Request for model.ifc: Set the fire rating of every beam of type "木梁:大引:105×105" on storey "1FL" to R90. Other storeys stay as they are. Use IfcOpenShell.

First a look at what the model holds.

```python
import ifcopenshell
import ifcopenshell.util.element

model = ifcopenshell.open("model.ifc")
print(model.schema)
storey = next(s for s in model.by_type("IfcBuildingStorey") if s.Name == "1FL")
beams = [e for e in ifcopenshell.util.element.get_decomposition(storey) if e.is_a("IfcBeam")]
seen = {}
for e in beams:
    element_type = ifcopenshell.util.element.get_type(e)
    key = (element_type.Name if element_type != e and element_type else None, ifcopenshell.util.element.get_pset(e, "Pset_BeamCommon", "FireRating"))
    seen[key] = seen.get(key, 0) + 1
for (name, value), count in sorted(seen.items(), key=str):
    print(count, "x", name, "|", value)
```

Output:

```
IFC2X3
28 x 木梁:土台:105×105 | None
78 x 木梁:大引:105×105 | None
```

```python
import ifcopenshell
import ifcopenshell.api.pset
import ifcopenshell.util.element

model = ifcopenshell.open("model.ifc")

storey = next(s for s in model.by_type("IfcBuildingStorey") if s.Name == "1FL")
beams = [e for e in ifcopenshell.util.element.get_decomposition(storey) if e.is_a("IfcBeam")]

count = 0
for e in beams:
    element_type = ifcopenshell.util.element.get_type(e)
    if element_type in (None, e) or element_type.Name != "木梁:大引:105×105":
        continue
    # add_pset returns the element's existing set when there is one.
    pset = ifcopenshell.api.pset.add_pset(model, product=e, name="Pset_BeamCommon")
    ifcopenshell.api.pset.edit_pset(model, pset=pset, properties={"FireRating": "R90"})
    count += 1

print(count, "beams updated")

model.write("model_v2.ifc")
```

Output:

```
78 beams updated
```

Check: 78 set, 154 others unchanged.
